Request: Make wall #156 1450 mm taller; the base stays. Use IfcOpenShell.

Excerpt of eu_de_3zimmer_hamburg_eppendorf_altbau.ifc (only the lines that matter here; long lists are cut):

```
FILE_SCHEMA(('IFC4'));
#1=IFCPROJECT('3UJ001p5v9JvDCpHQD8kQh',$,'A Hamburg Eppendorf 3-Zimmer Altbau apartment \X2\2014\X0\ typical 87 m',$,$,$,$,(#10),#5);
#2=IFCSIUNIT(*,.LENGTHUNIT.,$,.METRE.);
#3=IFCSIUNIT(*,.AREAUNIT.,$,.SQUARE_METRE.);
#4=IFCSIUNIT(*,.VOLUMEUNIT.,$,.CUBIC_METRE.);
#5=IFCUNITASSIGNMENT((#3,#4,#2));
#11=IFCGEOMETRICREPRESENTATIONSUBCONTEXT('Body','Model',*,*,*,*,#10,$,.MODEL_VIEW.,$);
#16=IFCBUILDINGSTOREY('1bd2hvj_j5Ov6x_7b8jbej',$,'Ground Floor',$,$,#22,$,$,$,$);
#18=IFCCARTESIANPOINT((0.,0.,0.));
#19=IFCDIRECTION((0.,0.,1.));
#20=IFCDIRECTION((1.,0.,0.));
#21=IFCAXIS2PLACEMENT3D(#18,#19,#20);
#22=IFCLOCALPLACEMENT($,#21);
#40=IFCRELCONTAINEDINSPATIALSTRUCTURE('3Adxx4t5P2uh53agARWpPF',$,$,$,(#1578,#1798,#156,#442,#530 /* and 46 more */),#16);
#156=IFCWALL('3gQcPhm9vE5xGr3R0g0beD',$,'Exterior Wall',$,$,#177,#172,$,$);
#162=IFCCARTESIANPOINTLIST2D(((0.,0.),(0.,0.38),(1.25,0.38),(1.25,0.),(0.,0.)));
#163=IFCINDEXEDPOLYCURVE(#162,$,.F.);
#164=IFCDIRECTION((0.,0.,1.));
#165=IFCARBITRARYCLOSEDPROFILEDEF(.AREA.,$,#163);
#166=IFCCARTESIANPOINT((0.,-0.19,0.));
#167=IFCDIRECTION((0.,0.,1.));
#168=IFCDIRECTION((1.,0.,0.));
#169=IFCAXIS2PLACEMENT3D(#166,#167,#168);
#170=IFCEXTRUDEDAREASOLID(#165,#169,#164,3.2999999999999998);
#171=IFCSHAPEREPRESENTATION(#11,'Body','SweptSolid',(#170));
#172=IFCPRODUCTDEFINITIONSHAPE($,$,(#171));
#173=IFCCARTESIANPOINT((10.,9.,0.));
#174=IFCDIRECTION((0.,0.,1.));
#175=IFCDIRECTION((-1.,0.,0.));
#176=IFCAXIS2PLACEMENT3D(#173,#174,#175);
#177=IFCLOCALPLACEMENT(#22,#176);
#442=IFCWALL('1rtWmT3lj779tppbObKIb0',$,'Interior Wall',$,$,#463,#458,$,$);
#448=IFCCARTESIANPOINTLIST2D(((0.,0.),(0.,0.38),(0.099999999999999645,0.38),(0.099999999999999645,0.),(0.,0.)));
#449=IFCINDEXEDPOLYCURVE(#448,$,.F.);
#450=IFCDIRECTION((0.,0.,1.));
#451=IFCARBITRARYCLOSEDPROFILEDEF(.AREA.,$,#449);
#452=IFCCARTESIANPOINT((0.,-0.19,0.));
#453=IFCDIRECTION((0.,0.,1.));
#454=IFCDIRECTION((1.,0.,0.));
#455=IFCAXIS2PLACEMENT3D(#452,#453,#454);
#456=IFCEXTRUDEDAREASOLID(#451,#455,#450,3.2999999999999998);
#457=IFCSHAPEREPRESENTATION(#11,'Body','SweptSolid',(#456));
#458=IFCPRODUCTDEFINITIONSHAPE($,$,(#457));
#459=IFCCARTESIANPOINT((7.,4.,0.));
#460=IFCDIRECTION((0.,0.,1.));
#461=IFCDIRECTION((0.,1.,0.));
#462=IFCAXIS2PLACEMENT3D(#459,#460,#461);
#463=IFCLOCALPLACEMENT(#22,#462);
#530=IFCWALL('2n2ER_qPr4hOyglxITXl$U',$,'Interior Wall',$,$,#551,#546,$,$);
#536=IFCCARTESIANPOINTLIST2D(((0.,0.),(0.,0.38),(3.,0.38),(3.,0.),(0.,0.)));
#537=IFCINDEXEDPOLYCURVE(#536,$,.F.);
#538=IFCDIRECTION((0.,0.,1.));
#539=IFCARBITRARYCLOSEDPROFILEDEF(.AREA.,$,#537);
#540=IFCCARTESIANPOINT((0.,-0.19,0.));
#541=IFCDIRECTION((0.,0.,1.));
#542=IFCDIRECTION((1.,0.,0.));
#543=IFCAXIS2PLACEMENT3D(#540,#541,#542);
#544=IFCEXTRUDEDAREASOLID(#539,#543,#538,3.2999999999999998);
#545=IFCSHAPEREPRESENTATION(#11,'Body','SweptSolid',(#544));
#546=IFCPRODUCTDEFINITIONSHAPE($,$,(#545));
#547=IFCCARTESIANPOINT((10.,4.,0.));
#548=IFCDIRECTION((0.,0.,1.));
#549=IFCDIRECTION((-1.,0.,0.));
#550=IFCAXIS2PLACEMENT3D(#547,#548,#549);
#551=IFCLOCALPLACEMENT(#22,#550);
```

```python
import ifcopenshell
import ifcopenshell.geom
import ifcopenshell.util.representation
import ifcopenshell.util.shape

model = ifcopenshell.open("eu_de_3zimmer_hamburg_eppendorf_altbau.ifc")
settings = ifcopenshell.geom.settings()


def volume(element):
    """Net volume in cubic metres, openings subtracted."""
    shape = ifcopenshell.geom.create_shape(settings, element)
    return ifcopenshell.util.shape.get_volume(shape.geometry)


wall = model.by_id(156)
before = volume(wall)

body = ifcopenshell.util.representation.get_representation(wall, "Model", "Body")
solid = body.Items[0]
old_height = solid.Depth
solid.Depth += 1.45
after = volume(wall)

print(f"height {old_height:g} -> {solid.Depth:g}, volume {before:.3f} -> {after:.3f} m3")

model.write("eu_de_3zimmer_hamburg_eppendorf_altbau_rev.ifc")
```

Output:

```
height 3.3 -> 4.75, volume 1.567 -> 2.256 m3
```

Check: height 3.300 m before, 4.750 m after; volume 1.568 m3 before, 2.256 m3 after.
